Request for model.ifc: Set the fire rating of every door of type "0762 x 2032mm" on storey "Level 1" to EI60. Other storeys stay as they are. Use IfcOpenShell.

First a look at what the model holds.

```python
import ifcopenshell
import ifcopenshell.util.element

model = ifcopenshell.open("model.ifc")
print(model.schema)
storey = next(s for s in model.by_type("IfcBuildingStorey") if s.Name == "Level 1")
doors = [e for e in ifcopenshell.util.element.get_decomposition(storey) if e.is_a("IfcDoor")]
seen = {}
for e in doors:
    element_type = ifcopenshell.util.element.get_type(e)
    key = (element_type.Name if element_type != e and element_type else None, ifcopenshell.util.element.get_pset(e, "Pset_DoorCommon", "FireRating"))
    seen[key] = seen.get(key, 0) + 1
for (name, value), count in sorted(seen.items(), key=str):
    print(count, "x", name, "|", value)
```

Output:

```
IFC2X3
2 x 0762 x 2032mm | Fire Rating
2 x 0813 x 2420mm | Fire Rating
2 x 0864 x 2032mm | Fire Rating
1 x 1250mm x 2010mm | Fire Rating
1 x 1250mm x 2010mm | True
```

```python
import ifcopenshell
import ifcopenshell.api.pset
import ifcopenshell.util.element

model = ifcopenshell.open("model.ifc")

storey = next(s for s in model.by_type("IfcBuildingStorey") if s.Name == "Level 1")
doors = [e for e in ifcopenshell.util.element.get_decomposition(storey) if e.is_a("IfcDoor")]

count = 0
for e in doors:
    element_type = ifcopenshell.util.element.get_type(e)
    if element_type in (None, e) or element_type.Name != "0762 x 2032mm":
        continue
    # add_pset returns the element's existing set when there is one.
    pset = ifcopenshell.api.pset.add_pset(model, product=e, name="Pset_DoorCommon")
    ifcopenshell.api.pset.edit_pset(model, pset=pset, properties={"FireRating": "EI60"})
    count += 1

print(count, "doors updated")

model.write("model_edited.ifc")
```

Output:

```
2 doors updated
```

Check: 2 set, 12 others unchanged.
